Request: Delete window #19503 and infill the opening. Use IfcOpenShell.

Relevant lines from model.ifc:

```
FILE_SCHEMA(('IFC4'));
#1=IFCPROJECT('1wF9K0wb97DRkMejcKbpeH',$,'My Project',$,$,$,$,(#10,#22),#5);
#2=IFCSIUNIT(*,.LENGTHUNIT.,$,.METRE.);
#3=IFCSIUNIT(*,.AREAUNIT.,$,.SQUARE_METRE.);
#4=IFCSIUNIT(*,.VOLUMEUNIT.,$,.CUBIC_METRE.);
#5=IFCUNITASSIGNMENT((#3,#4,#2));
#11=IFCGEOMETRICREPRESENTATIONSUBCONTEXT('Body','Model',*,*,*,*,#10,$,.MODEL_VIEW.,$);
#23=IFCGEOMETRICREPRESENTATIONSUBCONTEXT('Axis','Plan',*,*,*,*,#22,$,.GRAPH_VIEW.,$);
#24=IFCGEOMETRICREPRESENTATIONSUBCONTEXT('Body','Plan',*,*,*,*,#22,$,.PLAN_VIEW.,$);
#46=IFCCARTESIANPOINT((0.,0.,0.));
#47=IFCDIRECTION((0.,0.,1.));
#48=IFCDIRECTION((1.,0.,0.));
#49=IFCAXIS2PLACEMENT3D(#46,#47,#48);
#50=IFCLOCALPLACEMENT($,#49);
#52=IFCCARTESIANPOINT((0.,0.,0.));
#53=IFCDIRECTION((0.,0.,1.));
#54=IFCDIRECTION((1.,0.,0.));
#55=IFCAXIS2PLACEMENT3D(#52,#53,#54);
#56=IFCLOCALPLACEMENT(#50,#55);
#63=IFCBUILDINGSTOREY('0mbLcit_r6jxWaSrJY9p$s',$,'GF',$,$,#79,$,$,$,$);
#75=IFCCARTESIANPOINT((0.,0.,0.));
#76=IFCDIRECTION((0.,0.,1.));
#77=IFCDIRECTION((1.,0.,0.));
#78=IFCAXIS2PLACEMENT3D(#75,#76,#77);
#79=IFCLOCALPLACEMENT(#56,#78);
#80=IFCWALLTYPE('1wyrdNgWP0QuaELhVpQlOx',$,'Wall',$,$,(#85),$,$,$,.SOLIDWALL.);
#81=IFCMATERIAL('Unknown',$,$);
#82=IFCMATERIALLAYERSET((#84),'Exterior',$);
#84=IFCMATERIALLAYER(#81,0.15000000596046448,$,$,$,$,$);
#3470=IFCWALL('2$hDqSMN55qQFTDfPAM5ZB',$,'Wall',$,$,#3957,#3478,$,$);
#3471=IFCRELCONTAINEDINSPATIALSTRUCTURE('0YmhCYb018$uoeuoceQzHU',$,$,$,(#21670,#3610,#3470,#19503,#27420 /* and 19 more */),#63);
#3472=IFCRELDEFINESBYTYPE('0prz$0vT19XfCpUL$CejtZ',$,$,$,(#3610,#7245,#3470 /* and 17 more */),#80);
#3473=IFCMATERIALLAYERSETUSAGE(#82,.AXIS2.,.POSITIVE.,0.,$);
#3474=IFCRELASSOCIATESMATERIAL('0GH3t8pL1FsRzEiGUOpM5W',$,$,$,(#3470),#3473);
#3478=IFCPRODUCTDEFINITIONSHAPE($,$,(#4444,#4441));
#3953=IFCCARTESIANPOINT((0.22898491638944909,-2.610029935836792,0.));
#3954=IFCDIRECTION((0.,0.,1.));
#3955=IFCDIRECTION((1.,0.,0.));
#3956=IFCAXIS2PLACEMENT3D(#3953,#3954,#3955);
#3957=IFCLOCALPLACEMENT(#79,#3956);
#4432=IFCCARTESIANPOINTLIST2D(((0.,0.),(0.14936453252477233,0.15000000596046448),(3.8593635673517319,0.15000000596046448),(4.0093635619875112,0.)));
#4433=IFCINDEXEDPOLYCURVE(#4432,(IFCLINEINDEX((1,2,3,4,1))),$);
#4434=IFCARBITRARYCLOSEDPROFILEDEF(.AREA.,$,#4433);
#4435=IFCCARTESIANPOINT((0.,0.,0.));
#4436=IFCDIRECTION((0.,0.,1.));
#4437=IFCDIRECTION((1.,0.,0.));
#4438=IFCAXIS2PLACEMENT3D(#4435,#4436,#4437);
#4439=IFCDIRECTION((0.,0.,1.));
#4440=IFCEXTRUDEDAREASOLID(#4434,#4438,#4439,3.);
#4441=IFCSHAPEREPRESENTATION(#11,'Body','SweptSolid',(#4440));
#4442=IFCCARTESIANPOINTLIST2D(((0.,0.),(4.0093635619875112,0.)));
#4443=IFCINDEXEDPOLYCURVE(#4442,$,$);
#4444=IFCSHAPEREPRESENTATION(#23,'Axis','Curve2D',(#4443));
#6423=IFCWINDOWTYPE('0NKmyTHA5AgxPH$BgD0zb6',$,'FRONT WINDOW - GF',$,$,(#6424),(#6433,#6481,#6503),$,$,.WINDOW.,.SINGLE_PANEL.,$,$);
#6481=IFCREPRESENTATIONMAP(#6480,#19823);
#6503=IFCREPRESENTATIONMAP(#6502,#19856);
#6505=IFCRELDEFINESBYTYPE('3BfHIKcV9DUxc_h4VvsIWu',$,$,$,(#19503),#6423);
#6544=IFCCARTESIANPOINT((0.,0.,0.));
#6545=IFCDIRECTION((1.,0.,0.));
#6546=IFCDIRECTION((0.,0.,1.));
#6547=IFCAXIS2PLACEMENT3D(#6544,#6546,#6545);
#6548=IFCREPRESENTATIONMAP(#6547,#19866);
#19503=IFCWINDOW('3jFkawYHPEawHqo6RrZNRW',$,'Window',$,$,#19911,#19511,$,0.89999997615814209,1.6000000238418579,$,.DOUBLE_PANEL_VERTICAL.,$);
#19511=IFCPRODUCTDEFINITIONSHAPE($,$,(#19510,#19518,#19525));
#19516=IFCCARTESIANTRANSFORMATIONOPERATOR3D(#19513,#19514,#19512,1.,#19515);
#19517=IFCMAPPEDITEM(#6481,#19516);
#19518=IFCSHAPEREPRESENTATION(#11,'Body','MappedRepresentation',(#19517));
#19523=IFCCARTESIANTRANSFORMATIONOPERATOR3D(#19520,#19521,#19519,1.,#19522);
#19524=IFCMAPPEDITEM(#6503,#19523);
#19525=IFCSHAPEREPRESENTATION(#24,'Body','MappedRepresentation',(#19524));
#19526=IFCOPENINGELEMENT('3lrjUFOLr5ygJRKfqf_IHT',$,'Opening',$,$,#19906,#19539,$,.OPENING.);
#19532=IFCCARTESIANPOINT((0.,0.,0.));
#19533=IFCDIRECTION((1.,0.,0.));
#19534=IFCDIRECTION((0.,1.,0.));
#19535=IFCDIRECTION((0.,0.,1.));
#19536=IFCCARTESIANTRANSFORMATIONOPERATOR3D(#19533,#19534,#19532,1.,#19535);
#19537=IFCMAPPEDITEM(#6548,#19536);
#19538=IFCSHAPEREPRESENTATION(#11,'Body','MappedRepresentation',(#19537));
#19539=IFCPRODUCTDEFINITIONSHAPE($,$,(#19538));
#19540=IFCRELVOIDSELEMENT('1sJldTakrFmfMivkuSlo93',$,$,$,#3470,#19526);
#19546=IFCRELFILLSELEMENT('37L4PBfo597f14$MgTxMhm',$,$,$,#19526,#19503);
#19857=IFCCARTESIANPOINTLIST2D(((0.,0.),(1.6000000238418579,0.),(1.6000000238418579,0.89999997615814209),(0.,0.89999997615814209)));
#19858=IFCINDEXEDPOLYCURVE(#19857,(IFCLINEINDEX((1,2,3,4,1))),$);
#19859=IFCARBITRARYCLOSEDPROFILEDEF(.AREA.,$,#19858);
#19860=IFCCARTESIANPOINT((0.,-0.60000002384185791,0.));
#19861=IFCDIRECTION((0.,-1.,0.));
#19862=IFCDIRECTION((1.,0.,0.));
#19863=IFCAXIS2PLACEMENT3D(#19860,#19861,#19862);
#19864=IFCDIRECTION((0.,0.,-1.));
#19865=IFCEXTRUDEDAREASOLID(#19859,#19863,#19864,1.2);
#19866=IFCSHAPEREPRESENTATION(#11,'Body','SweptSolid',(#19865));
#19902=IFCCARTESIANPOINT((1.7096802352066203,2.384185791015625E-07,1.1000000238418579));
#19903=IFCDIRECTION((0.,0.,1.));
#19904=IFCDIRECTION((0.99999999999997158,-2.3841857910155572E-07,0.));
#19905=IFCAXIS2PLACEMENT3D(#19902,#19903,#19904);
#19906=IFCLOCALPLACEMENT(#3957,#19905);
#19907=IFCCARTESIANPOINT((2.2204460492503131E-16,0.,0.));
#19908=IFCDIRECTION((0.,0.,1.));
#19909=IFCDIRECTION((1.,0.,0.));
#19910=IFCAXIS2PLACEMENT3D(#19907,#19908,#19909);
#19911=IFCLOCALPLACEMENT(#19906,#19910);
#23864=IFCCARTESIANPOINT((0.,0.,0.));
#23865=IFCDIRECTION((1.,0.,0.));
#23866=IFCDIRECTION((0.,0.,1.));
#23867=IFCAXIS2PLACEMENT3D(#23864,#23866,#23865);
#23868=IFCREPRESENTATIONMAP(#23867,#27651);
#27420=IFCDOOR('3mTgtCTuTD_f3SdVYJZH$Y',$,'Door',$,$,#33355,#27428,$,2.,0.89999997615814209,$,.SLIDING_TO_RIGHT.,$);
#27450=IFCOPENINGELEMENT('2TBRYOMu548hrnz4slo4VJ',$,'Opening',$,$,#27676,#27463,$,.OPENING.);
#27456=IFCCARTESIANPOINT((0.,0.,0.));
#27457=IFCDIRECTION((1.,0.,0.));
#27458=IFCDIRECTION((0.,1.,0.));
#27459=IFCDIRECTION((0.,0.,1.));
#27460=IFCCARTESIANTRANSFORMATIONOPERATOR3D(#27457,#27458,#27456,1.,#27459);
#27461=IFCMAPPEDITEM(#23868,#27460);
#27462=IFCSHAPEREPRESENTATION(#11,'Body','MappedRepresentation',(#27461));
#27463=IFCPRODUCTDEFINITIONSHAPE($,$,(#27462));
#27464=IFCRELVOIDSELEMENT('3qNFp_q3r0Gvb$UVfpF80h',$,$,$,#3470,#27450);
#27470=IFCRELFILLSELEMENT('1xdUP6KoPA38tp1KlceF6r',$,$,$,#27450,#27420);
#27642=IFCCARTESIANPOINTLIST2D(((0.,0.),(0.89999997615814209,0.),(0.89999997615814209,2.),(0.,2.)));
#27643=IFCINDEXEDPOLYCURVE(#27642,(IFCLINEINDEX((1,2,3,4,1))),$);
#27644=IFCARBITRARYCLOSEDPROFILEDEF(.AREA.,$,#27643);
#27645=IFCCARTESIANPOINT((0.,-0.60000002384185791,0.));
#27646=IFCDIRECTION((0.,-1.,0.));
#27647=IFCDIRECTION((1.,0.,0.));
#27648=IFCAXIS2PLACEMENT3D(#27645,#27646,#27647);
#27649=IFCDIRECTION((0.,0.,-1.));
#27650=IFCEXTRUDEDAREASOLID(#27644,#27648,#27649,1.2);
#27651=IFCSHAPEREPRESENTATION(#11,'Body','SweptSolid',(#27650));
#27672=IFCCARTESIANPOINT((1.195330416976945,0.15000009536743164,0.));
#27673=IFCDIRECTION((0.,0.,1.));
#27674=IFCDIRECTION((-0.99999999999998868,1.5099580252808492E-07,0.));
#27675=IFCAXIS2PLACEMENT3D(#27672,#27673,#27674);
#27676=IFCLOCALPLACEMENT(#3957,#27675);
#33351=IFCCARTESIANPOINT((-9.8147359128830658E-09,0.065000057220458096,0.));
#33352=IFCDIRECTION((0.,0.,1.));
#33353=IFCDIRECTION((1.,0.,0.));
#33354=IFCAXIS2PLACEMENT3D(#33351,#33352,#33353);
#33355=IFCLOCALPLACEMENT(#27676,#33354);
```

```python
import ifcopenshell
import ifcopenshell.api.feature
import ifcopenshell.api.root
import ifcopenshell.geom
import ifcopenshell.util.shape

model = ifcopenshell.open("model.ifc")
settings = ifcopenshell.geom.settings()


def volume(element):
    """Net volume in cubic metres, openings subtracted."""
    shape = ifcopenshell.geom.create_shape(settings, element)
    return ifcopenshell.util.shape.get_volume(shape.geometry)


window = model.by_guid("3jFkawYHPEawHqo6RrZNRW")
opening = window.FillsVoids[0].RelatingOpeningElement
wall = opening.VoidsElements[0].RelatingBuildingElement
before = volume(wall)

ifcopenshell.api.root.remove_product(model, product=window)
ifcopenshell.api.feature.remove_feature(model, feature=opening)

after = volume(wall)

print(f"wall volume {before:.3f} -> {after:.3f} m3")

model.write("model_v2.ifc")
```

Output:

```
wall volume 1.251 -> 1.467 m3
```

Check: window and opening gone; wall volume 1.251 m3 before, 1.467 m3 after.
